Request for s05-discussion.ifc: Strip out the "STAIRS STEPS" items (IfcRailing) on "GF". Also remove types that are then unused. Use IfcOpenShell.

First a look at what the model holds.

```python
import ifcopenshell
import ifcopenshell.util.element

model = ifcopenshell.open("s05-discussion.ifc")
print(model.schema)
storey = next(s for s in model.by_type("IfcBuildingStorey") if s.Name == "GF")
railings = [e for e in ifcopenshell.util.element.get_decomposition(storey) if e.is_a("IfcRailing")]
seen = {}
for e in railings:
    element_type = ifcopenshell.util.element.get_type(e)
    name = element_type.Name if element_type not in (None, e) else None
    seen[name] = seen.get(name, 0) + 1
for name, count in sorted(seen.items(), key=str):
    print(count, "x", name)
```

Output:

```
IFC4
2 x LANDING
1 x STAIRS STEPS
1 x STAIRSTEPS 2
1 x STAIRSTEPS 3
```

```python
import ifcopenshell
import ifcopenshell.api.root
import ifcopenshell.util.element

model = ifcopenshell.open("s05-discussion.ifc")

storey = next(s for s in model.by_type("IfcBuildingStorey") if s.Name == "GF")
railings = [e for e in ifcopenshell.util.element.get_decomposition(storey) if e.is_a("IfcRailing")]
targets = [e for e in railings if (t := ifcopenshell.util.element.get_type(e)) not in (None, e) and t.Name == "STAIRS STEPS"]
types = {ifcopenshell.util.element.get_type(e) for e in targets} - {None, *targets}

for e in targets:
    ifcopenshell.api.root.remove_product(model, product=e)
print(len(targets), "removed")

unused = [t for t in types if not ifcopenshell.util.element.get_types(t)]
for t in unused:
    ifcopenshell.api.root.remove_product(model, product=t)
print(len(unused), "unused types removed")

model.write("s05-discussion-out.ifc")
```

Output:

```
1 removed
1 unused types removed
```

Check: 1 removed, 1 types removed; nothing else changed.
